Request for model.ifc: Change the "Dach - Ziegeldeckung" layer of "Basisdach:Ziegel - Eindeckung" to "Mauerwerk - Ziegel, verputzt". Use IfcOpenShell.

First a look at what the model holds.

```python
import ifcopenshell
import ifcopenshell.util.element

model = ifcopenshell.open("model.ifc")
print(model.schema)
for layer_set in model.by_type("IfcMaterialLayerSet"):
    if layer_set.LayerSetName == "Basisdach:Ziegel - Eindeckung":
        for layer in layer_set.MaterialLayers:
            print(layer.id(), layer.Material and layer.Material.Name, layer.LayerThickness, sep=" | ")
        print(len(ifcopenshell.util.element.get_elements_by_material(model, layer_set)), "elements and types use it")
print(sorted(m.Name for m in model.by_type("IfcMaterial") if m.Name)[:60])
```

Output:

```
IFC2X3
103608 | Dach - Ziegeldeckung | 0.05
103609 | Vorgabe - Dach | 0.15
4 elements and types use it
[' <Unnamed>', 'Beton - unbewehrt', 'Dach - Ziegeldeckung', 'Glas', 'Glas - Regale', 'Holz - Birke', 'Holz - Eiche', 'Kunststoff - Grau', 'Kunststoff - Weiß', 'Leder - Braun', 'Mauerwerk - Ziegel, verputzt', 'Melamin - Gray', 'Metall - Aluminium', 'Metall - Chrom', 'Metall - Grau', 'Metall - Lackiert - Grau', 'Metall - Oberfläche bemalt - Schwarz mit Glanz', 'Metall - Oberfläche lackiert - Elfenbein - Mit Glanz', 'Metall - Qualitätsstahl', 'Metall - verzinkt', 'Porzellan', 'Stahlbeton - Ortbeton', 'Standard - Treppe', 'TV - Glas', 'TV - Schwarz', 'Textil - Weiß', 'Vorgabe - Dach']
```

```python
import ifcopenshell
import ifcopenshell.api.material

model = ifcopenshell.open("model.ifc")

layer_set = next(s for s in model.by_type("IfcMaterialLayerSet") if s.LayerSetName == "Basisdach:Ziegel - Eindeckung")
layer = next(l for l in layer_set.MaterialLayers if l.Material and l.Material.Name == "Dach - Ziegeldeckung")
material = next(m for m in model.by_type("IfcMaterial") if m.Name == "Mauerwerk - Ziegel, verputzt")

# Point this one layer at the other material; renaming the old one would change it everywhere.
ifcopenshell.api.material.edit_layer(model, layer=layer, attributes={}, material=material)

print([l.Material.Name if l.Material else None for l in layer_set.MaterialLayers])

model.write("model_updated.ifc")
```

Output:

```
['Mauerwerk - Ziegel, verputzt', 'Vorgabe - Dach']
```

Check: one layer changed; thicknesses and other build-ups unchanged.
